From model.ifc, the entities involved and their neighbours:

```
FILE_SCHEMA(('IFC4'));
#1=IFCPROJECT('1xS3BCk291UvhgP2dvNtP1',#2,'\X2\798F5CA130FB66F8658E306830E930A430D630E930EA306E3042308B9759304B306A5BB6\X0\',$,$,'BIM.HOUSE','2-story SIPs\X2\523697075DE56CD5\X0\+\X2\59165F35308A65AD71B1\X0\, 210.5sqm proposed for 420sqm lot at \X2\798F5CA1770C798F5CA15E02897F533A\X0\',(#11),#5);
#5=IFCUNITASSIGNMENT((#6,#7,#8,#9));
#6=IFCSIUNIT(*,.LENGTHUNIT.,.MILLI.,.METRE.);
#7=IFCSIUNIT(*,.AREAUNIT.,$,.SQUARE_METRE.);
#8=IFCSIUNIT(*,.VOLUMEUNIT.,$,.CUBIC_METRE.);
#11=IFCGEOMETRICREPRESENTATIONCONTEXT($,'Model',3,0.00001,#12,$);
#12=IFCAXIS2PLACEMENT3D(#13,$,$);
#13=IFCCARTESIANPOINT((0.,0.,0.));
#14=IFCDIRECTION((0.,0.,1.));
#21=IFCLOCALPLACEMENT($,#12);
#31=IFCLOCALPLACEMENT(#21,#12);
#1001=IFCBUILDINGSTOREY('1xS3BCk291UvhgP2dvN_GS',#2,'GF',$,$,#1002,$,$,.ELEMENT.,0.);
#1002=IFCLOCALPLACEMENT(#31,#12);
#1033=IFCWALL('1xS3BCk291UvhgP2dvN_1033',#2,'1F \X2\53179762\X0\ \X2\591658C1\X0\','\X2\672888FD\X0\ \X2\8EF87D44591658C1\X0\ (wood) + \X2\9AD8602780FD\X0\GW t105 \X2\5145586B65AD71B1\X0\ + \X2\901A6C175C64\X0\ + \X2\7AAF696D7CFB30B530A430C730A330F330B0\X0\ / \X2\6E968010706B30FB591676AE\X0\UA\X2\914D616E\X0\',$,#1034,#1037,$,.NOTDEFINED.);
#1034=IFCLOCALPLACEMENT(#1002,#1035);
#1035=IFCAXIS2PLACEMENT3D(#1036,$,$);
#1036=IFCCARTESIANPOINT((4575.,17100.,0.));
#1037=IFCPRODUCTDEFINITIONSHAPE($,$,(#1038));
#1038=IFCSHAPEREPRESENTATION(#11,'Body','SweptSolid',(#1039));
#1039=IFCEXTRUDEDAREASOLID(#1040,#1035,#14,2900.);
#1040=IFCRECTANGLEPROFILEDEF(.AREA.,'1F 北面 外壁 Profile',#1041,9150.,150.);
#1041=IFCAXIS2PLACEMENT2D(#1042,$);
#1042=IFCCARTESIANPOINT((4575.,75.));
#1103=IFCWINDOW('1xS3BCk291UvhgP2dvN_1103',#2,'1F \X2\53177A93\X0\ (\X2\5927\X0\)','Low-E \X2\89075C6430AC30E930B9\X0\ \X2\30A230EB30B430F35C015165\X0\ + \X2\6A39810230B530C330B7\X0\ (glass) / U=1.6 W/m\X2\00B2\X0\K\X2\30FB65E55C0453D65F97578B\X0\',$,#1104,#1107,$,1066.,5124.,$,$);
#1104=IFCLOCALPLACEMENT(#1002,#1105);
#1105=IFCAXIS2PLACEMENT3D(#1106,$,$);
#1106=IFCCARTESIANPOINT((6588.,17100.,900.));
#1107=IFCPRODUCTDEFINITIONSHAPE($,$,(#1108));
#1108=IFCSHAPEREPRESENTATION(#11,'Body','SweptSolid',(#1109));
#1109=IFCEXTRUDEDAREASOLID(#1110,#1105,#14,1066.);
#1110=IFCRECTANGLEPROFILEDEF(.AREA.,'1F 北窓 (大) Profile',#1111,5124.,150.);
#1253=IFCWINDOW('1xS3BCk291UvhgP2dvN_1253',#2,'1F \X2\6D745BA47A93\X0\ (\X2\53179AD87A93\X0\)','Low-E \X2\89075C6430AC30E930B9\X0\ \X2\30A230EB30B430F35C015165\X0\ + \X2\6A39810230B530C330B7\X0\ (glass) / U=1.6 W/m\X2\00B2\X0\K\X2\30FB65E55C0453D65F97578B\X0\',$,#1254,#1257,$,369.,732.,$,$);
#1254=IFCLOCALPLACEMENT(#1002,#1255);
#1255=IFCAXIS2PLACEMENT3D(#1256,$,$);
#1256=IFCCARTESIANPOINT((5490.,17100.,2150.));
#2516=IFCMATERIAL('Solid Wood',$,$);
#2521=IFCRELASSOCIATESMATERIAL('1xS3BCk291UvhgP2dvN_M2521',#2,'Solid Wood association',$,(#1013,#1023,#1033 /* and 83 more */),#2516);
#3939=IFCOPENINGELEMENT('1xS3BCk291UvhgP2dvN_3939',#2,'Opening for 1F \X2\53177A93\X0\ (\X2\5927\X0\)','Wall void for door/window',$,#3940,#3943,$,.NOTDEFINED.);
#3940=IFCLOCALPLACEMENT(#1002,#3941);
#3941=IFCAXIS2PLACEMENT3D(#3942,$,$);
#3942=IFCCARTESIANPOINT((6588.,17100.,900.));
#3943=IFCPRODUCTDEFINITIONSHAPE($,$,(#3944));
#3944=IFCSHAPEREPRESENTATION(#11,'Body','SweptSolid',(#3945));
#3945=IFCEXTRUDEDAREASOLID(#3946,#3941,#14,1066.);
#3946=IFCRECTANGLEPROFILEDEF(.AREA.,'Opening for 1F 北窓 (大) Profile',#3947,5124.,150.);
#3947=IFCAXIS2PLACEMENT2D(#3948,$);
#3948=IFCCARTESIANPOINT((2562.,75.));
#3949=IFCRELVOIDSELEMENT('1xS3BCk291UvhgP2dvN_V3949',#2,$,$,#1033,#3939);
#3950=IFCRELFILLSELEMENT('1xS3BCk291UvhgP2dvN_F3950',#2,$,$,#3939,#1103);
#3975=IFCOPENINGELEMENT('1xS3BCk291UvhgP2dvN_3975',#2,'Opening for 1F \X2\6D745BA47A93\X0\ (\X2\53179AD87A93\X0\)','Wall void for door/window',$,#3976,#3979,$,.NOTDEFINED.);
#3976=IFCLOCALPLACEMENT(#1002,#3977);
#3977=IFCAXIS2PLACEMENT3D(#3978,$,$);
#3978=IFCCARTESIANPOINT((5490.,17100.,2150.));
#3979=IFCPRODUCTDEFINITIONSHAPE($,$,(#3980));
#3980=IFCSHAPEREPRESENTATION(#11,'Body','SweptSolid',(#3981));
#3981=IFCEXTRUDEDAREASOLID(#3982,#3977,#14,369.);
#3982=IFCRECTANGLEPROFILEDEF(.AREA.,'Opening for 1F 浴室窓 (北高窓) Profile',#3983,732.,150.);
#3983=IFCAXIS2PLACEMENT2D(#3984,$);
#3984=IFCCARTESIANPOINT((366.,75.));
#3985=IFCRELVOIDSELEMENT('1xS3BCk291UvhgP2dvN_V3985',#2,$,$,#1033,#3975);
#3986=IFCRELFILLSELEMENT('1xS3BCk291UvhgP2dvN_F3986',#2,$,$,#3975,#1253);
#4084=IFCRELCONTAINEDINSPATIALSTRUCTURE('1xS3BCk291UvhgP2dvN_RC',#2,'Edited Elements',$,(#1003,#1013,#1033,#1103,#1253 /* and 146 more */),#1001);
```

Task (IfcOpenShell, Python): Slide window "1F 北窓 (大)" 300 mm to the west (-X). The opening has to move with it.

```python
import ifcopenshell
import ifcopenshell.api.geometry
import ifcopenshell.util.placement

model = ifcopenshell.open("model.ifc")

window = model.by_guid("1xS3BCk291UvhgP2dvN_1103")
opening = window.FillsVoids[0].RelatingOpeningElement
wall = opening.VoidsElements[0].RelatingBuildingElement

wall_matrix = ifcopenshell.util.placement.get_local_placement(wall.ObjectPlacement)
shift = wall_matrix[:3, 0] * -300.0
before = ifcopenshell.util.placement.get_local_placement(window.ObjectPlacement)[:3, 3].copy()

# The window is not placed relative to its opening, so move both.
for product in (opening, window):
    matrix = ifcopenshell.util.placement.get_local_placement(product.ObjectPlacement)
    matrix[:3, 3] += shift
    ifcopenshell.api.geometry.edit_object_placement(model, product=product, matrix=matrix, is_si=False)

after = ifcopenshell.util.placement.get_local_placement(window.ObjectPlacement)[:3, 3]
print("window moved by", (after - before).round(3) + 0.0)

model.write("model-out.ifc")
```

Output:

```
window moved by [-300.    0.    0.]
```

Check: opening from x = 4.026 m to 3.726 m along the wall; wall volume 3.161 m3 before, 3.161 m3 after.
